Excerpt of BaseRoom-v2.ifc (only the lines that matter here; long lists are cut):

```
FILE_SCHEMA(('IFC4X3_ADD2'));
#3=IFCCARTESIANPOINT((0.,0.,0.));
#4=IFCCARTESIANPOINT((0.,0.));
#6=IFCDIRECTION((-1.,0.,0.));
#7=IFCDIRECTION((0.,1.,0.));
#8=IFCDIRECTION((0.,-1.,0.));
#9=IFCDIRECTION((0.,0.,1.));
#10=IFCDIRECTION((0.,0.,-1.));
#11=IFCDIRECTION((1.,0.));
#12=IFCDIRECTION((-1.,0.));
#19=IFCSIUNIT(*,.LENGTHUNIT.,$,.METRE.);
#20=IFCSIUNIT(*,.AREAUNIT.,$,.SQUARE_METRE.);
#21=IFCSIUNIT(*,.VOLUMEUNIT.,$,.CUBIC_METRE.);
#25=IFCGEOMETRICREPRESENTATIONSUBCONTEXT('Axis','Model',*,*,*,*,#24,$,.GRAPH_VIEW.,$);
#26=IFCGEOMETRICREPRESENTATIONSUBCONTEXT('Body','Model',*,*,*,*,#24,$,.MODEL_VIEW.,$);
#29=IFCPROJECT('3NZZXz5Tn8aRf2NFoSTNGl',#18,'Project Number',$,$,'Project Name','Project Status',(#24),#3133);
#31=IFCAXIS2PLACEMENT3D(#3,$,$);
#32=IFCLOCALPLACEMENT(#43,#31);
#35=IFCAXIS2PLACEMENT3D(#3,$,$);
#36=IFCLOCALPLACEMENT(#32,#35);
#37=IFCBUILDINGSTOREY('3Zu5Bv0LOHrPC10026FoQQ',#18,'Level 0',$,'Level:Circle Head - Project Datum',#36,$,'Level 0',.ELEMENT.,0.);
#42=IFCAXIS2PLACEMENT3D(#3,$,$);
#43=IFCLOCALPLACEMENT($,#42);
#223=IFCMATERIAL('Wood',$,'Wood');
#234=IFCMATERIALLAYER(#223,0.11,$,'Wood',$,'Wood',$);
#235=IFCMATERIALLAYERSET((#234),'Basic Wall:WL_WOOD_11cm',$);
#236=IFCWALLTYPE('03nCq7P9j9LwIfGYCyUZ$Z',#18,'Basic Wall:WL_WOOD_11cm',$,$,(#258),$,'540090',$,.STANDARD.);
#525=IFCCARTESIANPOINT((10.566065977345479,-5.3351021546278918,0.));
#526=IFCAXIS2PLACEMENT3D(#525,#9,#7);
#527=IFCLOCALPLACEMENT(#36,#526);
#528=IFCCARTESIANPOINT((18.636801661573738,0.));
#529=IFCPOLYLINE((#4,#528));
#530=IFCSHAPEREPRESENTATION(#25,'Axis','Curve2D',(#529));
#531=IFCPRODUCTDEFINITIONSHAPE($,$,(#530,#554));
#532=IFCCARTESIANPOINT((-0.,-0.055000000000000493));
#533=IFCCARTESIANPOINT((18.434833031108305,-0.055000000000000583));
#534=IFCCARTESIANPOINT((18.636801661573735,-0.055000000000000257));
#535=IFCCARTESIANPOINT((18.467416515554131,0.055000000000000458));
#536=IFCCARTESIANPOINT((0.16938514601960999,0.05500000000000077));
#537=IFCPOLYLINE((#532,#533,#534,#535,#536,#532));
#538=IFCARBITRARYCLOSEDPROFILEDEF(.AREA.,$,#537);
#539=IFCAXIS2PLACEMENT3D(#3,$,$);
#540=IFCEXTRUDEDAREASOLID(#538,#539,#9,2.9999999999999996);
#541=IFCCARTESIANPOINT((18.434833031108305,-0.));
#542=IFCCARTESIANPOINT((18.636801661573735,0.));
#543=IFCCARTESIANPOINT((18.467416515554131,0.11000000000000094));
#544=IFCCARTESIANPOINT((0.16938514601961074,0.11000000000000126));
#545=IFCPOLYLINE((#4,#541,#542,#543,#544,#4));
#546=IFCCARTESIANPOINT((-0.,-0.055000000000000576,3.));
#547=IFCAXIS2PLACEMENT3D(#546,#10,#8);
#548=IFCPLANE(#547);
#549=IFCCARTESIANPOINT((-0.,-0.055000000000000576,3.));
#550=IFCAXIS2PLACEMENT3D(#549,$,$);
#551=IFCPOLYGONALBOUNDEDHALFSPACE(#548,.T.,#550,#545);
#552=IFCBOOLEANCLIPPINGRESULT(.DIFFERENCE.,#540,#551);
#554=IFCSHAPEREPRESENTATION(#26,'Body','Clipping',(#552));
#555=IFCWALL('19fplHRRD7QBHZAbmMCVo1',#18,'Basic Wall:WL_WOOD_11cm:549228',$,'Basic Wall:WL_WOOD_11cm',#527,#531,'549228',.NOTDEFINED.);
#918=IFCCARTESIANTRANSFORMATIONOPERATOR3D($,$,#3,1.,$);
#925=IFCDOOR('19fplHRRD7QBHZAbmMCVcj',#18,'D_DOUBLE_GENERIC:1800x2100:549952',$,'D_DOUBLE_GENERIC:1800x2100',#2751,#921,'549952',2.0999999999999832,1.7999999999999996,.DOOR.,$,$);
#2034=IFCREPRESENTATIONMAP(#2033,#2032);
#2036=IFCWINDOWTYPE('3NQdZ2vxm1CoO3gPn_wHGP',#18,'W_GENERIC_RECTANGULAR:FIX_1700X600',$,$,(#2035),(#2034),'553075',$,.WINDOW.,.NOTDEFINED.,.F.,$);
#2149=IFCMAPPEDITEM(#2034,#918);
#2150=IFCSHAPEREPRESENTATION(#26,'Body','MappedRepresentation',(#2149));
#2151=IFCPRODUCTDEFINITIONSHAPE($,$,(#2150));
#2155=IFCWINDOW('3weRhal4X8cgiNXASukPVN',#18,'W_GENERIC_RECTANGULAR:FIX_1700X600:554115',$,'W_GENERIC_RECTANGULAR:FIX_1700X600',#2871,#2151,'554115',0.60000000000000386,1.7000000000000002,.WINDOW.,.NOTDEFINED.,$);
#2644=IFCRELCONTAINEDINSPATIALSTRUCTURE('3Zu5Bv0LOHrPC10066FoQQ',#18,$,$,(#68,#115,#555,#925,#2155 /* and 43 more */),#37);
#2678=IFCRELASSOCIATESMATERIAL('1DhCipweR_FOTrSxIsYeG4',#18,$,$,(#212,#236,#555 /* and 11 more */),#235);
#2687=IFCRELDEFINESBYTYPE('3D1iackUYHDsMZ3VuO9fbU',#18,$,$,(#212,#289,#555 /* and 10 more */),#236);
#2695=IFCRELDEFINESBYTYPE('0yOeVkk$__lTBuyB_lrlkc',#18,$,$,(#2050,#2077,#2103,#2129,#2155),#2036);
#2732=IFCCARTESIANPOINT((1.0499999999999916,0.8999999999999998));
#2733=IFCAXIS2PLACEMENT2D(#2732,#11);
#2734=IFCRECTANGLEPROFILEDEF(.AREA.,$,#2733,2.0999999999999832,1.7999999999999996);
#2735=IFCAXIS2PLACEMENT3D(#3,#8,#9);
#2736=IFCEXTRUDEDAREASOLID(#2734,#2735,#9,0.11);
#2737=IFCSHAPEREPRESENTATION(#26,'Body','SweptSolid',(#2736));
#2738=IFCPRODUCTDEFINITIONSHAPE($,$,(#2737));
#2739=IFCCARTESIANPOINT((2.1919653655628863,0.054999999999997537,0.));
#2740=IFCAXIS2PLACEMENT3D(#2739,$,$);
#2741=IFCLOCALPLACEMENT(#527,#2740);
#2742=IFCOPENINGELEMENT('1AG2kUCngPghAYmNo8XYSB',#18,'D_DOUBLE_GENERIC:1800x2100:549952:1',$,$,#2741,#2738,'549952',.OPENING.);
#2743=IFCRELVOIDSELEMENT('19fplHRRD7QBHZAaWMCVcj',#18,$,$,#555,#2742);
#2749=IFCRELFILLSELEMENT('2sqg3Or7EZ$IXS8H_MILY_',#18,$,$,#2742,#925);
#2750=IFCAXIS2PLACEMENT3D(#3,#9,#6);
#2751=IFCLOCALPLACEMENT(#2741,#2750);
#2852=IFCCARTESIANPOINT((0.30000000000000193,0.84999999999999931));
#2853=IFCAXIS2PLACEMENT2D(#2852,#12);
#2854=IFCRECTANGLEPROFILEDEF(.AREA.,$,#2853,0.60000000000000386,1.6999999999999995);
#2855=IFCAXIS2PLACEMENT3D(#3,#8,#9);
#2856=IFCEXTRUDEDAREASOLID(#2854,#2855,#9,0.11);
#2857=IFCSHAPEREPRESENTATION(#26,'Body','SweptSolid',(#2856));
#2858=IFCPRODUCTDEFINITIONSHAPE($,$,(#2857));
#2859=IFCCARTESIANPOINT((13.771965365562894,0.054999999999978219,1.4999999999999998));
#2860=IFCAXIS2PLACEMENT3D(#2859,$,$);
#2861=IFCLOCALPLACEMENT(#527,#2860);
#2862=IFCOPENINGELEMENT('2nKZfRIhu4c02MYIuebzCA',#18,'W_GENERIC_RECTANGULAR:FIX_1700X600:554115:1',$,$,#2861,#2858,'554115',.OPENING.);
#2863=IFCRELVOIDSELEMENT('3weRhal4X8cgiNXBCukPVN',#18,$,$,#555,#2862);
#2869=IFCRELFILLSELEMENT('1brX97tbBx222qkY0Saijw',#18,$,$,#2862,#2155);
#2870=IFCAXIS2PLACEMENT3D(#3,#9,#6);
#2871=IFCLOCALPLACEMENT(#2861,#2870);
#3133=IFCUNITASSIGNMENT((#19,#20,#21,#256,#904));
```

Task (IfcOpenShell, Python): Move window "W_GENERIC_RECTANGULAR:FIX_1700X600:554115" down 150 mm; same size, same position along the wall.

```python
import numpy as np
import ifcopenshell
import ifcopenshell.api.geometry
import ifcopenshell.util.placement
import ifcopenshell.util.unit

model = ifcopenshell.open("BaseRoom-v2.ifc")
unit_scale = ifcopenshell.util.unit.calculate_unit_scale(model)

window = model.by_id(2155)
opening = window.FillsVoids[0].RelatingOpeningElement
dz = -0.15

shift = np.array([0.0, 0.0, dz])
# The window is placed relative to its opening, so it follows when the opening moves.
matrix = ifcopenshell.util.placement.get_local_placement(opening.ObjectPlacement)
matrix[:3, 3] += shift
ifcopenshell.api.geometry.edit_object_placement(
    model, product=opening, matrix=matrix, is_si=False, should_transform_children=True
)

print(f"moved by {dz * unit_scale:+.3f} m")

model.write("BaseRoom-v2_edited.ifc")
```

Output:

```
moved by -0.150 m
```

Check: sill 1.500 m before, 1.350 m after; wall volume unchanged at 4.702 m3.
